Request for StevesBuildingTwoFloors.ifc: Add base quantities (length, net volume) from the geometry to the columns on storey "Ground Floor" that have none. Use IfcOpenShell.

First a look at what the model holds.

```python
import ifcopenshell
import ifcopenshell.util.element
import ifcopenshell.util.unit

model = ifcopenshell.open("StevesBuildingTwoFloors.ifc")
print(model.schema)
for unit_type in ("LENGTHUNIT", "AREAUNIT", "VOLUMEUNIT"):
    print(unit_type, ifcopenshell.util.unit.calculate_unit_scale(model, unit_type))
storey = next(s for s in model.by_type("IfcBuildingStorey") if s.Name == "Ground Floor")
columns = [e for e in ifcopenshell.util.element.get_decomposition(storey) if e.is_a("IfcColumn")]
for e in sorted(columns, key=lambda e: e.id()):
    print(e.id(), e.is_a(), e.Name, list(ifcopenshell.util.element.get_psets(e, qtos_only=True)), sep=" | ")
```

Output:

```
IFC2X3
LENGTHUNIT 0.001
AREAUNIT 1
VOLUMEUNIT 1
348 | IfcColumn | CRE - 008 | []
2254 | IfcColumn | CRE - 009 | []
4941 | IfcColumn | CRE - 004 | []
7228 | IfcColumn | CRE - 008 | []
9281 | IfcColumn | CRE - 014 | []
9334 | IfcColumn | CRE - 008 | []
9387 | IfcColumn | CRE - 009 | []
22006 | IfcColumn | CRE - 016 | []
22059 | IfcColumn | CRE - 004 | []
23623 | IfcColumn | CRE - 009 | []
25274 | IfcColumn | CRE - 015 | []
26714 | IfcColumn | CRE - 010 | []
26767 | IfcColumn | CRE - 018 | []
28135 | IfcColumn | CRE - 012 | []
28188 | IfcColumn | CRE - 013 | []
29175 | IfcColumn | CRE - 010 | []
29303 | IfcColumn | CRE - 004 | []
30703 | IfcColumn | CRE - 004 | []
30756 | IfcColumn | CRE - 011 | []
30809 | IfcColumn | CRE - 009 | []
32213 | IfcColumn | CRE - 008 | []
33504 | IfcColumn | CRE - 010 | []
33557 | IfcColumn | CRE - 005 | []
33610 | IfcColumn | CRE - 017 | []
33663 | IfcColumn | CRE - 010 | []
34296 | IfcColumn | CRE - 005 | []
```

```python
import ifcopenshell
import ifcopenshell.api.pset
import ifcopenshell.geom
import ifcopenshell.util.element
import ifcopenshell.util.shape
import ifcopenshell.util.unit

model = ifcopenshell.open("StevesBuildingTwoFloors.ifc")
unit_scale = ifcopenshell.util.unit.calculate_unit_scale(model)
volume_scale = ifcopenshell.util.unit.calculate_unit_scale(model, "VOLUMEUNIT")
settings = ifcopenshell.geom.settings()

storey = next(s for s in model.by_type("IfcBuildingStorey") if s.Name == "Ground Floor")
columns = [e for e in ifcopenshell.util.element.get_decomposition(storey) if e.is_a("IfcColumn")]

for e in sorted(columns, key=lambda e: e.id()):
    if ifcopenshell.util.element.get_psets(e, qtos_only=True, should_inherit=False):
        continue
    # Geometry comes back in metres, in the element's own axes.
    shape = ifcopenshell.geom.create_shape(settings, e)
    values = {
        "Length": ifcopenshell.util.shape.get_z(shape.geometry) / unit_scale,
        "NetVolume": ifcopenshell.util.shape.get_volume(shape.geometry) / volume_scale,
    }
    qto = ifcopenshell.api.pset.add_qto(model, product=e, name="BaseQuantities")
    ifcopenshell.api.pset.edit_qto(model, qto=qto, properties=values)
    print(e.id(), {k: round(v, 3) for k, v in values.items()})

model.write("StevesBuildingTwoFloors_edited.ifc")
```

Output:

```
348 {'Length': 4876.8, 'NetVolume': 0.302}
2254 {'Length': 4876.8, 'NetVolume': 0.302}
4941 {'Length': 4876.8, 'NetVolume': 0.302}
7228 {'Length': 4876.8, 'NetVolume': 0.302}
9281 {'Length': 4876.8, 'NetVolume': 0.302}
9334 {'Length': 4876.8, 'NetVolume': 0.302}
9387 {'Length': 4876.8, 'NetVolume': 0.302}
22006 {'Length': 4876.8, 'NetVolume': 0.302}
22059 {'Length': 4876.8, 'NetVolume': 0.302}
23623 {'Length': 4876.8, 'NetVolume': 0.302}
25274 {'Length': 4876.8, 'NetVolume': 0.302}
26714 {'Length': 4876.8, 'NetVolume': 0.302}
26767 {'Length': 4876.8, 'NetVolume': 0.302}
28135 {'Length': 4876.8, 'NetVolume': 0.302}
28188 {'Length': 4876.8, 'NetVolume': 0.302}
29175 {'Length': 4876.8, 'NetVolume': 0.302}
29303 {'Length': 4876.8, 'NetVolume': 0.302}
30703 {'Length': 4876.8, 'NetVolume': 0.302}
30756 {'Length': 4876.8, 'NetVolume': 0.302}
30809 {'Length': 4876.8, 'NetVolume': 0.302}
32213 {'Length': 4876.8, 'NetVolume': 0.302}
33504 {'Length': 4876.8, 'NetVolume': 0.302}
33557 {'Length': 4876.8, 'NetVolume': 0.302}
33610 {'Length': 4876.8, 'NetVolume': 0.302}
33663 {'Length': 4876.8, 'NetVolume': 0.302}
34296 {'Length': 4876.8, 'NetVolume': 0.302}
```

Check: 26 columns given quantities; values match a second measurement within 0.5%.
